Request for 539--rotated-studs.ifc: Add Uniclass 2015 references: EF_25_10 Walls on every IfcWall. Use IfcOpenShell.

First a look at what the model holds.

```python
import ifcopenshell

model = ifcopenshell.open("539--rotated-studs.ifc")
print(model.schema)
print("classifications:", [c.Name for c in model.by_type("IfcClassification")])
for ifc_class in ("IfcDoor", "IfcRoof", "IfcStair", "IfcWall", "IfcWindow"):
    print(ifc_class, len(model.by_type(ifc_class)))
```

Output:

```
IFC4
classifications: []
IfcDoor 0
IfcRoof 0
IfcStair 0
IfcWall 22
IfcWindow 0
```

```python
import ifcopenshell
import ifcopenshell.api.classification

model = ifcopenshell.open("539--rotated-studs.ifc")

system = ifcopenshell.api.classification.add_classification(model, classification="Uniclass 2015")

codes = {
    "IfcWall": ("EF_25_10", "Walls"),
}
for ifc_class, (code, name) in codes.items():
    products = model.by_type(ifc_class)
    ifcopenshell.api.classification.add_reference(
        model, products=products, classification=system, identification=code, name=name
    )
    print(code, len(products))

model.write("539--rotated-studs_rev.ifc")
```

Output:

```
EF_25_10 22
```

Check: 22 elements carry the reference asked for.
